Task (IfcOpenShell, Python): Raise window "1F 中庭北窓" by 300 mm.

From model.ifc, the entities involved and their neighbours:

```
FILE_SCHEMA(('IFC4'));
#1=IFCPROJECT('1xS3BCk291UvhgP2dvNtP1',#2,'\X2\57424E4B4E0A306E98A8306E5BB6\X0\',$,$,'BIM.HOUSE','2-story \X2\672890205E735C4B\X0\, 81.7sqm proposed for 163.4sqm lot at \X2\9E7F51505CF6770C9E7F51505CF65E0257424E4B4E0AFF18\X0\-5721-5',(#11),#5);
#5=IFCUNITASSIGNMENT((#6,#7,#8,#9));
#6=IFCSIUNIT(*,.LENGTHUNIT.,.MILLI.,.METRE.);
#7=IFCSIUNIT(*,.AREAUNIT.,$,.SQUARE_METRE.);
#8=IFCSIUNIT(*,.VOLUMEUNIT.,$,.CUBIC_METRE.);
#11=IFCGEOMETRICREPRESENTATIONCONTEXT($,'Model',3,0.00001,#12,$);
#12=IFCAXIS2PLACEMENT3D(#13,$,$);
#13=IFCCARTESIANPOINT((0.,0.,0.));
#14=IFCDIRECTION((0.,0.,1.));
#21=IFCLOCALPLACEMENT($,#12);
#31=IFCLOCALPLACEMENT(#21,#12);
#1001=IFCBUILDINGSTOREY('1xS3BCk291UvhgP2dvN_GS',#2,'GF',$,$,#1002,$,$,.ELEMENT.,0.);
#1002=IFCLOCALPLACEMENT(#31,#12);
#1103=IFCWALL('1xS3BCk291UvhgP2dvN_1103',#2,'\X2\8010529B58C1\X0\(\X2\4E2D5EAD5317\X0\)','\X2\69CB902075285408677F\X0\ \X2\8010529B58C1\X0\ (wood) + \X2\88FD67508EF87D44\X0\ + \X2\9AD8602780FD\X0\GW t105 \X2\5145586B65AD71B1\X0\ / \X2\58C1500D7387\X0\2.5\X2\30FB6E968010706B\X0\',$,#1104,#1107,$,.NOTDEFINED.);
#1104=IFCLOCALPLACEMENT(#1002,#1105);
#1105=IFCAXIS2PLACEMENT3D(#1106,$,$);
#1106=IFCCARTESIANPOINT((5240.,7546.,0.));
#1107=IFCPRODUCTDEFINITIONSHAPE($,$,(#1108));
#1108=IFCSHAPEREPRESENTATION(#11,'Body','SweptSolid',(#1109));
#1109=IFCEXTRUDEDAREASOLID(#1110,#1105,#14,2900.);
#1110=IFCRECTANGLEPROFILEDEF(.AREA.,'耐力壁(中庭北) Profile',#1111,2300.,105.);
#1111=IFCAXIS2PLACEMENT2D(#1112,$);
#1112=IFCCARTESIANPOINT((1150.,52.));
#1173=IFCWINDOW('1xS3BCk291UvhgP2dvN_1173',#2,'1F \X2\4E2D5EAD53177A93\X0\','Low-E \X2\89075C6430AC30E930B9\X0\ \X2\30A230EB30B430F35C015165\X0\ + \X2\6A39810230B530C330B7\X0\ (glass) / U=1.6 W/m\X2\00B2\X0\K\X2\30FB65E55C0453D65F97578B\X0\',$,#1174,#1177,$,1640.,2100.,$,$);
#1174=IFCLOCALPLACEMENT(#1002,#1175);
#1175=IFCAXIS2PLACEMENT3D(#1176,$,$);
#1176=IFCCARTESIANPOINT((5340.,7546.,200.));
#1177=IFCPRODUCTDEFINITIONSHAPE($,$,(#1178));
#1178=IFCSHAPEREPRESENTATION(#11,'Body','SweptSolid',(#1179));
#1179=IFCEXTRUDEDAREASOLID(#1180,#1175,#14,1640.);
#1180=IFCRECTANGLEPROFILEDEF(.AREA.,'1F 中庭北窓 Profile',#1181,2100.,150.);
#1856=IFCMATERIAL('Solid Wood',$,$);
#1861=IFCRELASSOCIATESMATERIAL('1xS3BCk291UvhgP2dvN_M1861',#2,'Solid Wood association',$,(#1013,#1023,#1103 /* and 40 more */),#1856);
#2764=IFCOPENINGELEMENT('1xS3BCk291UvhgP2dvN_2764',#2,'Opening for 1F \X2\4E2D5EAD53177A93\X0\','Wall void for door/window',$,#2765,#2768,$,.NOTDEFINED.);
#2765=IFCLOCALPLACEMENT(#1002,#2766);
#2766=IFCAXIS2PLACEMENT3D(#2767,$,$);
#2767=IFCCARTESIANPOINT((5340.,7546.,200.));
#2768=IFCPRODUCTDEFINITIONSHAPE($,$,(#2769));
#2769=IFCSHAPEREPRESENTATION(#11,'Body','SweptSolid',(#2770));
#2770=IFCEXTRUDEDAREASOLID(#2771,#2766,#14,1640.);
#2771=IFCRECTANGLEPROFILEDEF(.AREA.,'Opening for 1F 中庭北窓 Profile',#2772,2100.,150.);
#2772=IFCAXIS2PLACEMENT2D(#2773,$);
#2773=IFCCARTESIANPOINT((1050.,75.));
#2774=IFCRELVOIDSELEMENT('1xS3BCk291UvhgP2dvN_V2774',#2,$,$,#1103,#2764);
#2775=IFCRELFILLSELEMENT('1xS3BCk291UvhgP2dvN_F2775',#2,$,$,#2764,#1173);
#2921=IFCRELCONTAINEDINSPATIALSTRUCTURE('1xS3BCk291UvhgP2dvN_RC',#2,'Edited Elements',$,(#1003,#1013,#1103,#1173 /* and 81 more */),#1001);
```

```python
import numpy as np
import ifcopenshell
import ifcopenshell.api.geometry
import ifcopenshell.util.placement
import ifcopenshell.util.unit

model = ifcopenshell.open("model.ifc")
unit_scale = ifcopenshell.util.unit.calculate_unit_scale(model)

window = model.by_id(1173)
opening = window.FillsVoids[0].RelatingOpeningElement
dz = 300.0

shift = np.array([0.0, 0.0, dz])
# The window is not placed relative to its opening, so move both.
for product in (opening, window):
    matrix = ifcopenshell.util.placement.get_local_placement(product.ObjectPlacement)
    matrix[:3, 3] += shift
    ifcopenshell.api.geometry.edit_object_placement(model, product=product, matrix=matrix, is_si=False)

print(f"moved by {dz * unit_scale:+.3f} m")

model.write("model_updated.ifc")
```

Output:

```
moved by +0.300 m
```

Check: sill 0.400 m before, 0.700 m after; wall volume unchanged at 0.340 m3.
